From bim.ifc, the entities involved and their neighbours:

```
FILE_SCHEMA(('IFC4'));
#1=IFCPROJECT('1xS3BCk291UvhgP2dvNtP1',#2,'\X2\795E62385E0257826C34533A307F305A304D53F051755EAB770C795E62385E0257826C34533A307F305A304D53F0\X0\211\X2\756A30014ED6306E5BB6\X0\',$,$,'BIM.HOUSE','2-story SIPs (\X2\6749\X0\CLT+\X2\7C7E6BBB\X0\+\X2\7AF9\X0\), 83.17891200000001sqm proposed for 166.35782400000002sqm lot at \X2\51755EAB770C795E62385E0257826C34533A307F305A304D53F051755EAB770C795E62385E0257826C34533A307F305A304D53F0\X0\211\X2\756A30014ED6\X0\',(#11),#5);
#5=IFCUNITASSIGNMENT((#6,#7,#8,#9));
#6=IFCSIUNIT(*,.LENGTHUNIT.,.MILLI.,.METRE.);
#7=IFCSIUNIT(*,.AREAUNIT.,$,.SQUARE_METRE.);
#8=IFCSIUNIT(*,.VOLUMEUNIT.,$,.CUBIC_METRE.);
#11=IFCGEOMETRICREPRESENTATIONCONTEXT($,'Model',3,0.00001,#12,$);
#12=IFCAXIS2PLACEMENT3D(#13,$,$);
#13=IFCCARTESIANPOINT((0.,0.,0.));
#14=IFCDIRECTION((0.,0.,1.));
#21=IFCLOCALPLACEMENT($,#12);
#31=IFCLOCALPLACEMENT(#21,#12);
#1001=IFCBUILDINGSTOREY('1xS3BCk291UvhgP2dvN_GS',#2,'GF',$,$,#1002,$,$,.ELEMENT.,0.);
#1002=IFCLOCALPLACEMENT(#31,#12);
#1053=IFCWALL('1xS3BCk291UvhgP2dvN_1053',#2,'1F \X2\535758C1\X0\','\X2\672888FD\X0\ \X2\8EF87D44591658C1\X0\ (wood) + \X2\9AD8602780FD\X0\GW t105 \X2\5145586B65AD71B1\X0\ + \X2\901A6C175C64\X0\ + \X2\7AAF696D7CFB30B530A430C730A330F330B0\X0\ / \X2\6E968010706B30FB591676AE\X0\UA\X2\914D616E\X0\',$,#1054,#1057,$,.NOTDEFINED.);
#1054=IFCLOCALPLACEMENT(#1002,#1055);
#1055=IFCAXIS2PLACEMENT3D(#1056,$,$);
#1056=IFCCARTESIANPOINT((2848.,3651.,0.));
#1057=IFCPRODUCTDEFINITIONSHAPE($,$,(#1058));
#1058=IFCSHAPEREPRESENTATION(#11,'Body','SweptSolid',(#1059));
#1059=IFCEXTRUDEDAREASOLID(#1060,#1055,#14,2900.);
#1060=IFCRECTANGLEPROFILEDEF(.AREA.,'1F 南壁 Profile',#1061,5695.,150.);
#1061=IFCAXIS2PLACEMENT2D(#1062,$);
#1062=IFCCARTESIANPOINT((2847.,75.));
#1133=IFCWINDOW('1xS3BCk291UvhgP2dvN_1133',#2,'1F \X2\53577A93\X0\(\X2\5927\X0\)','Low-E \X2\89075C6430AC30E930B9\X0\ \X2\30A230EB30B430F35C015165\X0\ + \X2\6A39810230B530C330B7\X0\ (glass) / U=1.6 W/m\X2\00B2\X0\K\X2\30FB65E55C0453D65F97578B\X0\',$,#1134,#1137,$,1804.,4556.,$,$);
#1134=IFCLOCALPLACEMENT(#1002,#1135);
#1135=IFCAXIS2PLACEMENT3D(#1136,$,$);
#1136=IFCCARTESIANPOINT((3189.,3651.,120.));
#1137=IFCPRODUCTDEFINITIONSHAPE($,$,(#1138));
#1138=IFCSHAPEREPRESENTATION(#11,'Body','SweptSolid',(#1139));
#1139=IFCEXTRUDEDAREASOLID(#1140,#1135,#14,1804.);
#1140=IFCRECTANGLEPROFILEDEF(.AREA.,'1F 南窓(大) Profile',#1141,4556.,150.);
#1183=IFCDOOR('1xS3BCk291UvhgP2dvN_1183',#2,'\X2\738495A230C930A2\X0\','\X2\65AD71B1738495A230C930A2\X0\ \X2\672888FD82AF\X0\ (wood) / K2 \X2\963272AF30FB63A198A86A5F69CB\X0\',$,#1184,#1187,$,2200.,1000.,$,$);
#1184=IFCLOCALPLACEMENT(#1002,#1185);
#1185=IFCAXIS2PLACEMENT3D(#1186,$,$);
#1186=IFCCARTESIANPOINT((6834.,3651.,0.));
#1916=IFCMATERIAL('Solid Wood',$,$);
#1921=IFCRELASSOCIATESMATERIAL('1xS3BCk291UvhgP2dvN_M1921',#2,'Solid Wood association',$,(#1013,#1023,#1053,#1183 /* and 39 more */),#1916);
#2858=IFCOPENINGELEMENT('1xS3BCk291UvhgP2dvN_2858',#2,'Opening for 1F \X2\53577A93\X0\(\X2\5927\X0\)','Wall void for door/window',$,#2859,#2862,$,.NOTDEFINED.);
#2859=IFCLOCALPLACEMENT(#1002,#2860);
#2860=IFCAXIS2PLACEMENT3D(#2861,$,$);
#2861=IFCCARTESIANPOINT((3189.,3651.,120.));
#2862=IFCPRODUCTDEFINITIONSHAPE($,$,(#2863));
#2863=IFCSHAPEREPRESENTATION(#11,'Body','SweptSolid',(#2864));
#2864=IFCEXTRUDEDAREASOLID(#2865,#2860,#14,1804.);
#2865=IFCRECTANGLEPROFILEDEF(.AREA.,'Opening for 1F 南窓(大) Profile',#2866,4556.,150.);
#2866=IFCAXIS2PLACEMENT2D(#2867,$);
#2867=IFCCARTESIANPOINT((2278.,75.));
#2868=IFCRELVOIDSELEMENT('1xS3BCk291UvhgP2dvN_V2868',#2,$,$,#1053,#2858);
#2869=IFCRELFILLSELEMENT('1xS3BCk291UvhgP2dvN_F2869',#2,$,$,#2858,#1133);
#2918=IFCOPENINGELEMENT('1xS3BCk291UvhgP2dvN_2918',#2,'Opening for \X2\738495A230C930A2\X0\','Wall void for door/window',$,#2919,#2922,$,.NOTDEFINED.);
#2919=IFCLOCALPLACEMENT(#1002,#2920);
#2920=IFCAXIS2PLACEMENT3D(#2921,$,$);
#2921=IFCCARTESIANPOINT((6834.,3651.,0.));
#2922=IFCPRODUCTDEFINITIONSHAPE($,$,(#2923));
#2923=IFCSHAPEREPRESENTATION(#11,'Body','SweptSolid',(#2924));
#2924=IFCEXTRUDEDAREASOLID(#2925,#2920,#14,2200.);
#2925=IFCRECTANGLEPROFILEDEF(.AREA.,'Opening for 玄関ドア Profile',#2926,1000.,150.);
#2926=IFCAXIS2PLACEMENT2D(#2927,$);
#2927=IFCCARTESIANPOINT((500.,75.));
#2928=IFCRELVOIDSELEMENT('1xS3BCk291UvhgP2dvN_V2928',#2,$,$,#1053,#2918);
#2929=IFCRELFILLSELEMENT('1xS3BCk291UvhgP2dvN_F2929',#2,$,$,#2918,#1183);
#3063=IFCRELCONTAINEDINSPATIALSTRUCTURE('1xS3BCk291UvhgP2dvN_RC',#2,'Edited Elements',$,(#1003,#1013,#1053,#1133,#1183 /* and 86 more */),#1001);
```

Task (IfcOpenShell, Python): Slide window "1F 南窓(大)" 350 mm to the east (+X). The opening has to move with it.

```python
import ifcopenshell
import ifcopenshell.api.geometry
import ifcopenshell.util.placement
import ifcopenshell.util.unit

model = ifcopenshell.open("bim.ifc")
unit_scale = ifcopenshell.util.unit.calculate_unit_scale(model)

window = model.by_guid("1xS3BCk291UvhgP2dvN_1133")
opening = window.FillsVoids[0].RelatingOpeningElement
wall = opening.VoidsElements[0].RelatingBuildingElement

wall_matrix = ifcopenshell.util.placement.get_local_placement(wall.ObjectPlacement)
shift = wall_matrix[:3, 0] * 0.35 / unit_scale
before = ifcopenshell.util.placement.get_local_placement(window.ObjectPlacement)[:3, 3].copy()

# The window is not placed relative to its opening, so move both.
for product in (opening, window):
    matrix = ifcopenshell.util.placement.get_local_placement(product.ObjectPlacement)
    matrix[:3, 3] += shift
    ifcopenshell.api.geometry.edit_object_placement(model, product=product, matrix=matrix, is_si=False)

after = ifcopenshell.util.placement.get_local_placement(window.ObjectPlacement)[:3, 3]
print("window moved by", (after - before).round(3) + 0.0)

model.write("bim_v2.ifc")
```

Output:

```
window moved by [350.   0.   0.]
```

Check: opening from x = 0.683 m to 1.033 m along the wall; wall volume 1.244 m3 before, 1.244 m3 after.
